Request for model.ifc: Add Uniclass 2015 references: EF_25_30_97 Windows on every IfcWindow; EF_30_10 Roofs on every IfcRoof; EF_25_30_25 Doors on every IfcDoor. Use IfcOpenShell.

First a look at what the model holds.

```python
import ifcopenshell

model = ifcopenshell.open("model.ifc")
print(model.schema)
print("classifications:", [c.Name for c in model.by_type("IfcClassification")])
for ifc_class in ("IfcDoor", "IfcRoof", "IfcStair", "IfcWall", "IfcWindow"):
    print(ifc_class, len(model.by_type(ifc_class)))
```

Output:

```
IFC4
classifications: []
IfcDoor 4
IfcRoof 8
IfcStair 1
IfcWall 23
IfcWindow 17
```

```python
import ifcopenshell
import ifcopenshell.api.classification

model = ifcopenshell.open("model.ifc")

system = ifcopenshell.api.classification.add_classification(model, classification="Uniclass 2015")

codes = {
    "IfcWindow": ("EF_25_30_97", "Windows"),
    "IfcRoof": ("EF_30_10", "Roofs"),
    "IfcDoor": ("EF_25_30_25", "Doors"),
}
for ifc_class, (code, name) in codes.items():
    products = model.by_type(ifc_class)
    ifcopenshell.api.classification.add_reference(
        model, products=products, classification=system, identification=code, name=name
    )
    print(code, len(products))

model.write("model-out.ifc")
```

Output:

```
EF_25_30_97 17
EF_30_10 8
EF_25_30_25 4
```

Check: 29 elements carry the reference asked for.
